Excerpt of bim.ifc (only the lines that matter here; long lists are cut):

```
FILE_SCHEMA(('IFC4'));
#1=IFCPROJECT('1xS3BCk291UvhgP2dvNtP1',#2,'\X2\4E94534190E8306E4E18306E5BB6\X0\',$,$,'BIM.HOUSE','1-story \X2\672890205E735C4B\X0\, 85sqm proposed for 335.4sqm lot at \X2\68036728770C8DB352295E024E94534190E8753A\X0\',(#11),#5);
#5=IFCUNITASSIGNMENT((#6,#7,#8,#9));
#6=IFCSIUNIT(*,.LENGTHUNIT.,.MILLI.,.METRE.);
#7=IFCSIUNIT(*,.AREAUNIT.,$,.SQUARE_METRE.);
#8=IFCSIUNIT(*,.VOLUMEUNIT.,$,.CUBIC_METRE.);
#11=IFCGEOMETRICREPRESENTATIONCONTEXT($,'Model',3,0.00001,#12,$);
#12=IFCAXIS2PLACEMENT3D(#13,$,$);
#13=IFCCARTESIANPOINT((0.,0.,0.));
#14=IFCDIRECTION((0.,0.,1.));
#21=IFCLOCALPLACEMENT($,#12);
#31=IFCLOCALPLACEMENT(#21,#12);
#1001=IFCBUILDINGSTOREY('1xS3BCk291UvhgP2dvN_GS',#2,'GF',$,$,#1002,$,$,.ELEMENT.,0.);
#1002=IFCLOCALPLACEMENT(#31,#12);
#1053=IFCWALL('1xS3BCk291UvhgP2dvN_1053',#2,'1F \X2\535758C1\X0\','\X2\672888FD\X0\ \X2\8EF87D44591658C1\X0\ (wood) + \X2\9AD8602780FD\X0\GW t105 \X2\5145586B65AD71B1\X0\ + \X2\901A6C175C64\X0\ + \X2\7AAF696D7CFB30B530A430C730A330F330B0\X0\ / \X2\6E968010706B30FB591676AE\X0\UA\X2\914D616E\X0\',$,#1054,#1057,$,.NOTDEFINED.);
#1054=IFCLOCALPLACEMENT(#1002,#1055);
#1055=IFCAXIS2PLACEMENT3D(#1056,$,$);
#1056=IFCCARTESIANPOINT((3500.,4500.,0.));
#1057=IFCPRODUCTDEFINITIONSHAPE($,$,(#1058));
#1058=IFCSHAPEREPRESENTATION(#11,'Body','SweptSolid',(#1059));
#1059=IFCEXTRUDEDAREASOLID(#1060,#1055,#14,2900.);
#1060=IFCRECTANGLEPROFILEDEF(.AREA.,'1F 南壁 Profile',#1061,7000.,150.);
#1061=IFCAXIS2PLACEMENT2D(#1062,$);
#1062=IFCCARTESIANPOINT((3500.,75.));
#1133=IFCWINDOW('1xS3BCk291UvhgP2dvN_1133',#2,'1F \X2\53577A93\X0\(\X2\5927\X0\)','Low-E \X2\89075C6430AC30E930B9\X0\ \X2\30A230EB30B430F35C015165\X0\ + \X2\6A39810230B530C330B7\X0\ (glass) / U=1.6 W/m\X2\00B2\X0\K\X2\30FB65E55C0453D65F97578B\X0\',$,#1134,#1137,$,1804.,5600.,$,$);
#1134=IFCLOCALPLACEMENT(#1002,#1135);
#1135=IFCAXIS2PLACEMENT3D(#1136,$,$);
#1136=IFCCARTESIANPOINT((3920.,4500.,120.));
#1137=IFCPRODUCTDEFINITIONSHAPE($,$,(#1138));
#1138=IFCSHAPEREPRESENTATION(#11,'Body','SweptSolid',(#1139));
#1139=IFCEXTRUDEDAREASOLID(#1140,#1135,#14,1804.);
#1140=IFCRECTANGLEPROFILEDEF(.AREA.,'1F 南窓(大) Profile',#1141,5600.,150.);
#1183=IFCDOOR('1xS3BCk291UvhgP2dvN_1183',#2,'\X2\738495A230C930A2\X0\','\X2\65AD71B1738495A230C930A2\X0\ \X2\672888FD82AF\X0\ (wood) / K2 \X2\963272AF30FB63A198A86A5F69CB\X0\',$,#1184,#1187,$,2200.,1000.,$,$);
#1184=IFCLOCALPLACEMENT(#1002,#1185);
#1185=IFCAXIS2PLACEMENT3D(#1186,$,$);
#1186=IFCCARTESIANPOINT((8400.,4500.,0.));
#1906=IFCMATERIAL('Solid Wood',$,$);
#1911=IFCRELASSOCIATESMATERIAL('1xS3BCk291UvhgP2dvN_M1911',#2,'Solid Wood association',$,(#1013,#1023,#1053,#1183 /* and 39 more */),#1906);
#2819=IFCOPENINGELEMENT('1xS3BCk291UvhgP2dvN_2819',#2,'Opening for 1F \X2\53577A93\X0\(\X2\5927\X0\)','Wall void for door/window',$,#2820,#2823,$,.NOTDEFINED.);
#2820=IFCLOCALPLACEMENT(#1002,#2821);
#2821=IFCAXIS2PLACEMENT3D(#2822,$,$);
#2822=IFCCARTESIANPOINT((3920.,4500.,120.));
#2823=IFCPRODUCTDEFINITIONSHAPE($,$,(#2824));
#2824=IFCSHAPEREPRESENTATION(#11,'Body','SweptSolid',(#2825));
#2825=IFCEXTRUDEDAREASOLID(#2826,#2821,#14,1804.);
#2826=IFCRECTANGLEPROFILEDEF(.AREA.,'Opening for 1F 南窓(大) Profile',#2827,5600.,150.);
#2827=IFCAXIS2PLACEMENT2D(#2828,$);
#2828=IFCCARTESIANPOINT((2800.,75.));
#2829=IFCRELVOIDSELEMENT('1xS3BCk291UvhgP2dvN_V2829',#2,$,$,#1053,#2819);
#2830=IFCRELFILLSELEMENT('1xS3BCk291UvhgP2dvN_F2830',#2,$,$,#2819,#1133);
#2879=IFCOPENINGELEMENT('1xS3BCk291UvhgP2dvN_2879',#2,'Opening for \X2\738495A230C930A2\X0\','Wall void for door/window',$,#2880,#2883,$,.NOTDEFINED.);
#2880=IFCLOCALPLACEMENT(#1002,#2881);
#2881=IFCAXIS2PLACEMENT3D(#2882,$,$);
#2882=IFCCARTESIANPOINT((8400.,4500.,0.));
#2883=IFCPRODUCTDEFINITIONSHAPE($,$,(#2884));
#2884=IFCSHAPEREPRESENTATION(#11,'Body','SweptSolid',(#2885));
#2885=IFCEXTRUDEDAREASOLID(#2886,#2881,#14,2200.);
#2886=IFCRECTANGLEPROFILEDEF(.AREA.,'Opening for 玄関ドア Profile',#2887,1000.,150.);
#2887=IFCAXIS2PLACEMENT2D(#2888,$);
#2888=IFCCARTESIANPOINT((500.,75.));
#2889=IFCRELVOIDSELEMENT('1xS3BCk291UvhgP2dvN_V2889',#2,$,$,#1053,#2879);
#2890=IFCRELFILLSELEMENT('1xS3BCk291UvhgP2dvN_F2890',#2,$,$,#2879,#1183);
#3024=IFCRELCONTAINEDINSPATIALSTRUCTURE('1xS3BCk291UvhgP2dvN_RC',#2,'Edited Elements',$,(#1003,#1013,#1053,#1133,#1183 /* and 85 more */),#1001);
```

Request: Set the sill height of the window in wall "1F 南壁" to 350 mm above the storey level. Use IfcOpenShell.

```python
import numpy as np
import ifcopenshell
import ifcopenshell.api.geometry
import ifcopenshell.geom
import ifcopenshell.util.element
import ifcopenshell.util.placement
import ifcopenshell.util.shape
import ifcopenshell.util.unit

model = ifcopenshell.open("bim.ifc")
unit_scale = ifcopenshell.util.unit.calculate_unit_scale(model)

window = model.by_guid("1xS3BCk291UvhgP2dvN_1133")
opening = window.FillsVoids[0].RelatingOpeningElement
storey = ifcopenshell.util.element.get_container(window, ifc_class="IfcBuildingStorey")
level = ifcopenshell.util.placement.get_local_placement(storey.ObjectPlacement)[2, 3]

# The opening's origin need not be at the sill, so measure its lowest point.
shape = ifcopenshell.geom.create_shape(ifcopenshell.geom.settings(), opening)
bottom = ifcopenshell.util.shape.get_shape_bottom_elevation(shape, shape.geometry) / unit_scale
dz = level + 0.35 / unit_scale - bottom

shift = np.array([0.0, 0.0, dz])
# The window is not placed relative to its opening, so move both.
for product in (opening, window):
    matrix = ifcopenshell.util.placement.get_local_placement(product.ObjectPlacement)
    matrix[:3, 3] += shift
    ifcopenshell.api.geometry.edit_object_placement(model, product=product, matrix=matrix, is_si=False)

print(f"moved by {dz * unit_scale:+.3f} m")

model.write("bim-out.ifc")
```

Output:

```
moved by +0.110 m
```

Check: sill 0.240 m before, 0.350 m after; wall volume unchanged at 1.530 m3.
